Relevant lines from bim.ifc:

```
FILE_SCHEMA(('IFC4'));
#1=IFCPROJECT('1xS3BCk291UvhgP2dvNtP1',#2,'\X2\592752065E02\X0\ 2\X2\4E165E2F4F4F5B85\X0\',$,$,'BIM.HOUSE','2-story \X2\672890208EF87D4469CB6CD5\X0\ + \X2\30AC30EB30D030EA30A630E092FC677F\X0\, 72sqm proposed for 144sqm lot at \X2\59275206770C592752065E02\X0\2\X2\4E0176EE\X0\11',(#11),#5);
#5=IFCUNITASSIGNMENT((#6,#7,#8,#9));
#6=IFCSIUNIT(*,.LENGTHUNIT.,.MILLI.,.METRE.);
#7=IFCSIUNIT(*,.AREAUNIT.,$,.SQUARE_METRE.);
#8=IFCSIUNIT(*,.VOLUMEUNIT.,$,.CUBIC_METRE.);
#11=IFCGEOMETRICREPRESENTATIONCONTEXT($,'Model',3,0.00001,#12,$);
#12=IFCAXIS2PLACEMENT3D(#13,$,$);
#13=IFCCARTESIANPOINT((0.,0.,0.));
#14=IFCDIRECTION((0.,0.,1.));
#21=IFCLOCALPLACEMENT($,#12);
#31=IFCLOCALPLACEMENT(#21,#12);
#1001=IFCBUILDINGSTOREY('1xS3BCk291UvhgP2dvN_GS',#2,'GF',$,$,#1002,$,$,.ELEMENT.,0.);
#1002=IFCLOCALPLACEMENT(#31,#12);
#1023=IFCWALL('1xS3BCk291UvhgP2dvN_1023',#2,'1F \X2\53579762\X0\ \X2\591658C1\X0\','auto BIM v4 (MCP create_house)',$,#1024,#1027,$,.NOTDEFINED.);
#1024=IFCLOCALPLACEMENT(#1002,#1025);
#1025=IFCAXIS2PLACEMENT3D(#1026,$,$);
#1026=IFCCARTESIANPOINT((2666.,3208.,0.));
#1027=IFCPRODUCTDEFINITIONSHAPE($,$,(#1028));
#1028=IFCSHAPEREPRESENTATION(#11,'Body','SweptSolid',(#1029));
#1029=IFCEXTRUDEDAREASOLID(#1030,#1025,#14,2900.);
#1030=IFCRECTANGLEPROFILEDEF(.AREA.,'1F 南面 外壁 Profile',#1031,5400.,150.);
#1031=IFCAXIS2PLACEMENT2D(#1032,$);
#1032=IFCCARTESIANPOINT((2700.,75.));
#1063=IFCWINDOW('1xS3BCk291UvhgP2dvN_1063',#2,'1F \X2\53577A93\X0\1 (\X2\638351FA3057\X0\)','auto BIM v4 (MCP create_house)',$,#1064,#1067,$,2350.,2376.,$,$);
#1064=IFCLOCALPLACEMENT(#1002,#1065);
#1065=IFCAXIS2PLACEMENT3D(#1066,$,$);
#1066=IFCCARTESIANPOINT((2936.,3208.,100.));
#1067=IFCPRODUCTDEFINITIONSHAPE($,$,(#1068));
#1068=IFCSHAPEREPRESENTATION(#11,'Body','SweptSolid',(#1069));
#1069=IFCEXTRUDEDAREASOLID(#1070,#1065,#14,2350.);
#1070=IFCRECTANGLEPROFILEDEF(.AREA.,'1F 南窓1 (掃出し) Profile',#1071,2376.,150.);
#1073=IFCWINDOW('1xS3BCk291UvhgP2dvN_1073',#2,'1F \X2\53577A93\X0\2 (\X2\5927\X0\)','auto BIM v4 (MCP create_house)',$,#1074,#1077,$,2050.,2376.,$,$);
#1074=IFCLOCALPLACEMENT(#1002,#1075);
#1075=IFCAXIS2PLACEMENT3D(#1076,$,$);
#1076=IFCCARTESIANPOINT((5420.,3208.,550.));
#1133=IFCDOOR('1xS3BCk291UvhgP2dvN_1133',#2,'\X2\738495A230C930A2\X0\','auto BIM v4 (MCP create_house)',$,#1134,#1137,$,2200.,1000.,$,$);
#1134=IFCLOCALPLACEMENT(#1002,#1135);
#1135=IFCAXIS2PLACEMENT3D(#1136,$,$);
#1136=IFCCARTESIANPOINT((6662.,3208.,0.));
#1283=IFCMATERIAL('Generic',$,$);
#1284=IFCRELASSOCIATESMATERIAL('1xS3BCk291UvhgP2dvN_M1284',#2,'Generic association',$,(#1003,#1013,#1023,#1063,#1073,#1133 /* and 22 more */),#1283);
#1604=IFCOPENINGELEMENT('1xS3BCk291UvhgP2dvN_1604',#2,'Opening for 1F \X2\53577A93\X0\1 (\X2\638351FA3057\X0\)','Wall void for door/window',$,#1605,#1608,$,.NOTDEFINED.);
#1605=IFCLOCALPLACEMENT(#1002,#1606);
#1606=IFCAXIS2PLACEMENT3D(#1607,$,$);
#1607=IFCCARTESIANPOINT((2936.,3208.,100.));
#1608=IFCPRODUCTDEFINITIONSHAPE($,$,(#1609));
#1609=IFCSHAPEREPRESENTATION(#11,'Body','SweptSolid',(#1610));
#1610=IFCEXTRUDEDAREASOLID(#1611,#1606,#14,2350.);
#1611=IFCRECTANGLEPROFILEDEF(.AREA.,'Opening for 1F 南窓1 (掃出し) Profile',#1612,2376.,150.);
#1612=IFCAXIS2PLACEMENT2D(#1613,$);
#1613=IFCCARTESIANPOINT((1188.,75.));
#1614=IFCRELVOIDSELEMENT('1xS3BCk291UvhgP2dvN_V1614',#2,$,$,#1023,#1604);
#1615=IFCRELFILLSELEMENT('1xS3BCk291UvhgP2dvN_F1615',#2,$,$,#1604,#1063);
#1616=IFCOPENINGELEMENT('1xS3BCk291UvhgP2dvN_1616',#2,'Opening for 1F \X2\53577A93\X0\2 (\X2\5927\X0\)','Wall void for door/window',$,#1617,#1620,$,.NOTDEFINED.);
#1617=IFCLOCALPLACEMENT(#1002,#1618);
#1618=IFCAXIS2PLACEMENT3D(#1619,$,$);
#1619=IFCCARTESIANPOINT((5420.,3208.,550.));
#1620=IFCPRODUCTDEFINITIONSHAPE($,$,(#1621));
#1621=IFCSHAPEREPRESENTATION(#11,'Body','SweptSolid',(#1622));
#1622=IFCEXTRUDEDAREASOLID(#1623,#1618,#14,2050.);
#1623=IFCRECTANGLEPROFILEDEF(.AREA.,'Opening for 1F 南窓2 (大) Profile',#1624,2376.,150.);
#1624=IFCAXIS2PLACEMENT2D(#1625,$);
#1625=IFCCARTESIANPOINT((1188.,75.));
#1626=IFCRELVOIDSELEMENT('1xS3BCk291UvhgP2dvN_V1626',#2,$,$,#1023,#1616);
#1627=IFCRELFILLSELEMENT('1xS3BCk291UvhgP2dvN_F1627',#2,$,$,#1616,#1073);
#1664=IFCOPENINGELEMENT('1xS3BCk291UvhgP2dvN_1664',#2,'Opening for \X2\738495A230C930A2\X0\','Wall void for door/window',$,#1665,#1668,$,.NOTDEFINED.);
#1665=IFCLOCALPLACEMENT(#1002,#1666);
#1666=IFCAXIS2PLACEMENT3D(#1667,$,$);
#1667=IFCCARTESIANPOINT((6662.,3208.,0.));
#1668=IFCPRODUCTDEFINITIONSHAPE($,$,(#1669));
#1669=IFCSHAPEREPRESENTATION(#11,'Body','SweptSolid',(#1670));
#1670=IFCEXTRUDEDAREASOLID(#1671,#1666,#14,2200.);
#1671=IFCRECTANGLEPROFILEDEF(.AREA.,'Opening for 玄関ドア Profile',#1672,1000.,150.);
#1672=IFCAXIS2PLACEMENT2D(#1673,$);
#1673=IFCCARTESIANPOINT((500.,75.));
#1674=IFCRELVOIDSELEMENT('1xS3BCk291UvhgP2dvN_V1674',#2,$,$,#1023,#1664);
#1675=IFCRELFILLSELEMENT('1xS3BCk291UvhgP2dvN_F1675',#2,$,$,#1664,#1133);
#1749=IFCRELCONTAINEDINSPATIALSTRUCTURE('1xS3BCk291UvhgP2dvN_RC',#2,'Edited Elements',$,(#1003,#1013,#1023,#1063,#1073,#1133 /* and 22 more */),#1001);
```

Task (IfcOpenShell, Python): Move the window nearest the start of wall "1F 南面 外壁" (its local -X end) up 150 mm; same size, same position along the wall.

```python
import numpy as np
import ifcopenshell
import ifcopenshell.api.geometry
import ifcopenshell.util.placement
import ifcopenshell.util.unit

model = ifcopenshell.open("bim.ifc")
unit_scale = ifcopenshell.util.unit.calculate_unit_scale(model)

window = model.by_guid("1xS3BCk291UvhgP2dvN_1063")
opening = window.FillsVoids[0].RelatingOpeningElement
dz = 0.15 / unit_scale

shift = np.array([0.0, 0.0, dz])
# The window is not placed relative to its opening, so move both.
for product in (opening, window):
    matrix = ifcopenshell.util.placement.get_local_placement(product.ObjectPlacement)
    matrix[:3, 3] += shift
    ifcopenshell.api.geometry.edit_object_placement(model, product=product, matrix=matrix, is_si=False)

print(f"moved by {dz * unit_scale:+.3f} m")

model.write("bim-out.ifc")
```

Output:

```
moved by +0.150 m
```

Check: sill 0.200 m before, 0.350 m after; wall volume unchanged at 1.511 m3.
